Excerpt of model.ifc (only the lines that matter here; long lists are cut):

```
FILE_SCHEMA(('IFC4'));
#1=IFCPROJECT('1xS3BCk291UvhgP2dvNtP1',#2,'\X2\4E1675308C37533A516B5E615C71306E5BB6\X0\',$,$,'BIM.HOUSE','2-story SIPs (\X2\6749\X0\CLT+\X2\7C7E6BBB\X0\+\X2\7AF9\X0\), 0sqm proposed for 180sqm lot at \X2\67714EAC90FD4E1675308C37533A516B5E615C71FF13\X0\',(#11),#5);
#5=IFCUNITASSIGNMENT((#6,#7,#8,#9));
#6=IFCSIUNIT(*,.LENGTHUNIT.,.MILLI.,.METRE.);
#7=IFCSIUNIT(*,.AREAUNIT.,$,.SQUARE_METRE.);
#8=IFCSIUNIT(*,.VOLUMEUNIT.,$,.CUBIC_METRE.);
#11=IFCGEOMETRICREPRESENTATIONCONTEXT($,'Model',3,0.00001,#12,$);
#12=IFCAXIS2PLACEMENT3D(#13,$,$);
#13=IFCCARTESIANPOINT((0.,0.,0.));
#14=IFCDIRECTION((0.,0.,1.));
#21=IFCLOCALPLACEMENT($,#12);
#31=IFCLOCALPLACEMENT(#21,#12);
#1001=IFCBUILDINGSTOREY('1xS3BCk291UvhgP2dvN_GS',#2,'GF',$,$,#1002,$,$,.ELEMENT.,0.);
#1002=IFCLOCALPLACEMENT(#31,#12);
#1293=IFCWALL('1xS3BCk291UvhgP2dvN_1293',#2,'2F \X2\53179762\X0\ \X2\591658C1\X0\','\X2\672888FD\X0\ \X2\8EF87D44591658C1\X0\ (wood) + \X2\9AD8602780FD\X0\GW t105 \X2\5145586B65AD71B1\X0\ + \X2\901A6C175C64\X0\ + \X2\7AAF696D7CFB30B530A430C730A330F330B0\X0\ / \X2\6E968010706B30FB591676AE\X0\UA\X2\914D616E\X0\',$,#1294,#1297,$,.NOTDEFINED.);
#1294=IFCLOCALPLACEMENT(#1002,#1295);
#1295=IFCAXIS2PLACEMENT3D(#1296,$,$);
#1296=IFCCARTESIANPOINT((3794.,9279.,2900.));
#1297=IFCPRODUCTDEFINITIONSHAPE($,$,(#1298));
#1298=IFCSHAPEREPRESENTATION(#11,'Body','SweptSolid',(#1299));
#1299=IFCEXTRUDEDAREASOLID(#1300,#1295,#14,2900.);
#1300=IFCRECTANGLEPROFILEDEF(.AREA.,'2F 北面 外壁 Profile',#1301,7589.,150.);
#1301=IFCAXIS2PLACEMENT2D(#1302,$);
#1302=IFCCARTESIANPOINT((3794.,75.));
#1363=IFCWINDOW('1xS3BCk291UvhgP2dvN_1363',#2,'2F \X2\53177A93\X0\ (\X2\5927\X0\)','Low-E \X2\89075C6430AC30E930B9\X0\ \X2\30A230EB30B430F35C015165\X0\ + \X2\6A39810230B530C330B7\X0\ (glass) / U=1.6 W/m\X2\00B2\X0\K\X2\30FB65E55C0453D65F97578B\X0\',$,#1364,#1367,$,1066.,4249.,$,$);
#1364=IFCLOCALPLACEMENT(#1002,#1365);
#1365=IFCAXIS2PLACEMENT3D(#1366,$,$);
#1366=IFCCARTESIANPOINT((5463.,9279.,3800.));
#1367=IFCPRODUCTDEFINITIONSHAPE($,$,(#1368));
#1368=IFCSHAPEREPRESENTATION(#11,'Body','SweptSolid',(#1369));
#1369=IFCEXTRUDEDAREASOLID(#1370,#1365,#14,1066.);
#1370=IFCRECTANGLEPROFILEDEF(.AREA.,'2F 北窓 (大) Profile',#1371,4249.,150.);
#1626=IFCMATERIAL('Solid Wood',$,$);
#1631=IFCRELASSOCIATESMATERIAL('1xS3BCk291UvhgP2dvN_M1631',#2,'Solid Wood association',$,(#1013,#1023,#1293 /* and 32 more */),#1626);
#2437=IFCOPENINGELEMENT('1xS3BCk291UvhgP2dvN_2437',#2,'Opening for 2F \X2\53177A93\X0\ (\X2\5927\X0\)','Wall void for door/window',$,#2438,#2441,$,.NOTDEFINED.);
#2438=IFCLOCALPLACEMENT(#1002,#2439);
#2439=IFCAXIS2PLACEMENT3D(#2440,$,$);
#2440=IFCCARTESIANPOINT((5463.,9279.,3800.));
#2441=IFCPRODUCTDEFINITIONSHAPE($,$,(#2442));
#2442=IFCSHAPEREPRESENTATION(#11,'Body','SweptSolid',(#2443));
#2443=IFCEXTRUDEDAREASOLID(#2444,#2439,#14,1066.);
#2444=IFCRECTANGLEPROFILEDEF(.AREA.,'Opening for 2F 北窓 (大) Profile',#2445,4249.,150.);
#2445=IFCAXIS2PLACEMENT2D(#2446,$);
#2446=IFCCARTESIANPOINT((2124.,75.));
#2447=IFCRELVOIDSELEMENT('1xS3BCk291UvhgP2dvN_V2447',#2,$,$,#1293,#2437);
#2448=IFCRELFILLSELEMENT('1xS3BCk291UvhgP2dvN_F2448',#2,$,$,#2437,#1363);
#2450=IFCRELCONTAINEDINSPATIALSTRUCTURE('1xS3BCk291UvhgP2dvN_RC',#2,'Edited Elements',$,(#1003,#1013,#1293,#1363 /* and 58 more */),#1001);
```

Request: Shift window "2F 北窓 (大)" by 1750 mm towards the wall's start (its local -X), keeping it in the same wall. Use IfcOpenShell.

```python
import ifcopenshell
import ifcopenshell.api.geometry
import ifcopenshell.util.placement
import ifcopenshell.util.unit

model = ifcopenshell.open("model.ifc")
unit_scale = ifcopenshell.util.unit.calculate_unit_scale(model)

window = model.by_guid("1xS3BCk291UvhgP2dvN_1363")
opening = window.FillsVoids[0].RelatingOpeningElement
wall = opening.VoidsElements[0].RelatingBuildingElement

wall_matrix = ifcopenshell.util.placement.get_local_placement(wall.ObjectPlacement)
shift = wall_matrix[:3, 0] * -1.75 / unit_scale
before = ifcopenshell.util.placement.get_local_placement(window.ObjectPlacement)[:3, 3].copy()

# The window is not placed relative to its opening, so move both.
for product in (opening, window):
    matrix = ifcopenshell.util.placement.get_local_placement(product.ObjectPlacement)
    matrix[:3, 3] += shift
    ifcopenshell.api.geometry.edit_object_placement(model, product=product, matrix=matrix, is_si=False)

after = ifcopenshell.util.placement.get_local_placement(window.ObjectPlacement)[:3, 3]
print("window moved by", (after - before).round(3) + 0.0)

model.write("model-out.ifc")
```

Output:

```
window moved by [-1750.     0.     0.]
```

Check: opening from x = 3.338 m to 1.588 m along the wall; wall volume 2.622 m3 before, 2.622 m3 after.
